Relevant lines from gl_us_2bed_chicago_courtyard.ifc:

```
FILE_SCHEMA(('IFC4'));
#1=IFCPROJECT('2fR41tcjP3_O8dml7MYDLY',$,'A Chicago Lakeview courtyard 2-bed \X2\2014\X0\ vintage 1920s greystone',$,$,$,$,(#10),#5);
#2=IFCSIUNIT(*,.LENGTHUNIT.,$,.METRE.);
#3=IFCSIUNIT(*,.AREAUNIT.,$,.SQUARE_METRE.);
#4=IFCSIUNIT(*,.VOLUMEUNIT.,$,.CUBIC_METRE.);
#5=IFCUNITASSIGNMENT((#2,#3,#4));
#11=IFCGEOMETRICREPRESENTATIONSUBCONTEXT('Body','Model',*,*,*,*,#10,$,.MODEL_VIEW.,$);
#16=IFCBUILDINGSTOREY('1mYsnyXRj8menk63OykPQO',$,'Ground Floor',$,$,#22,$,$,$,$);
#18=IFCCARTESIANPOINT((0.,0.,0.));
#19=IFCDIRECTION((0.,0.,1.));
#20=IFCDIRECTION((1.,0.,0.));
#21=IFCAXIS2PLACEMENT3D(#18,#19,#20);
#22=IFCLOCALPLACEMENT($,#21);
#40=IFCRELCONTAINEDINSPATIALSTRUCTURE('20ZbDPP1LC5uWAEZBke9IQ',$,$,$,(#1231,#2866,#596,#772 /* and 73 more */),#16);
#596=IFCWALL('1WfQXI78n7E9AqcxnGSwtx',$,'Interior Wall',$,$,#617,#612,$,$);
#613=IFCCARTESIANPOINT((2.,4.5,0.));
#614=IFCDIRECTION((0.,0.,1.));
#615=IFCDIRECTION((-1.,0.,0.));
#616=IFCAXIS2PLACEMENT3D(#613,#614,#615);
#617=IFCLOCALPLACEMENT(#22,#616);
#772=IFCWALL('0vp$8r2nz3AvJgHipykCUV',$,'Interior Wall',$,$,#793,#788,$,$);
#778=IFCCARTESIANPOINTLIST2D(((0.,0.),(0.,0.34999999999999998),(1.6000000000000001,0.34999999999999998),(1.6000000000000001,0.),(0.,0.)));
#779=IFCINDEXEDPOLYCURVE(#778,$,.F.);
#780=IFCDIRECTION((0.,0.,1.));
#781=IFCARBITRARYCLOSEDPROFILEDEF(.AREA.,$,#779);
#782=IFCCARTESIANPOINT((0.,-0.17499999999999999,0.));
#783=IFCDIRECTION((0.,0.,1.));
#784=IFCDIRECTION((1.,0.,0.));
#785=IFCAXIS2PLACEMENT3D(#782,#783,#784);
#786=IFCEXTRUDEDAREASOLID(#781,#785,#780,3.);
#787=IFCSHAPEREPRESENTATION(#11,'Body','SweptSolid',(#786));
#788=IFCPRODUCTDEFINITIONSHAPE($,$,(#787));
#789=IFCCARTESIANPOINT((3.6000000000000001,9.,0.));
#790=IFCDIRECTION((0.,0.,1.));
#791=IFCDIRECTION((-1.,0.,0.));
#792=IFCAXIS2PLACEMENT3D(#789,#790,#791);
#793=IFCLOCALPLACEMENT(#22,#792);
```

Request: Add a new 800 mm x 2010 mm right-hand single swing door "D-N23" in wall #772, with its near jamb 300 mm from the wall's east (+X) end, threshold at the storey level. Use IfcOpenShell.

```python
import numpy as np
import ifcopenshell
import ifcopenshell.api.feature
import ifcopenshell.api.geometry
import ifcopenshell.api.root
import ifcopenshell.api.spatial
import ifcopenshell.geom
import ifcopenshell.util.element
import ifcopenshell.util.placement
import ifcopenshell.util.representation
import ifcopenshell.util.shape
import ifcopenshell.util.unit

model = ifcopenshell.open("gl_us_2bed_chicago_courtyard.ifc")
unit_scale = ifcopenshell.util.unit.calculate_unit_scale(model)
settings = ifcopenshell.geom.settings()


def volume(element):
    """Net volume in cubic metres, openings subtracted."""
    shape = ifcopenshell.geom.create_shape(settings, element)
    return ifcopenshell.util.shape.get_volume(shape.geometry)


wall = model.by_guid("0vp$8r2nz3AvJgHipykCUV")
storey = ifcopenshell.util.element.get_container(wall, ifc_class="IfcBuildingStorey")
context = ifcopenshell.util.representation.get_context(model, "Model", "Body", "MODEL_VIEW")
before = volume(wall)

width, height, from_end, sill = 0.8, 2.01, 0.3, 0.0  # metres

# The wall runs along its own X axis, and the end named is its -X end.
wall_shape = ifcopenshell.geom.create_shape(settings, wall)
x, y, z = ifcopenshell.util.shape.get_vertices(wall_shape.geometry).T
start = x.min() + from_end
face, thickness = float(y.min()), float(y.max() - y.min())
wall_matrix = ifcopenshell.util.placement.get_local_placement(wall.ObjectPlacement)
level = ifcopenshell.util.placement.get_local_placement(storey.ObjectPlacement)[2, 3]


def in_wall(x, y):
    """Placement at x, y metres in the wall's axes, at sill height."""
    matrix = wall_matrix.copy()
    matrix[:, 3] = wall_matrix @ np.array([x / unit_scale, y / unit_scale, 0.0, 1.0])
    matrix[2, 3] = level + sill / unit_scale
    return matrix


# Opening: a box that overshoots both wall faces by 50 mm.
opening = ifcopenshell.api.root.create_entity(model, ifc_class="IfcOpeningElement", predefined_type="OPENING")
box = ifcopenshell.api.geometry.add_wall_representation(
    model, context=context, length=width, height=height, thickness=thickness + 0.1
)
ifcopenshell.api.geometry.assign_representation(model, product=opening, representation=box)
ifcopenshell.api.geometry.edit_object_placement(model, product=opening, matrix=in_wall(start, face - 0.05), is_si=False)
ifcopenshell.api.feature.add_feature(model, feature=opening, element=wall)

door = ifcopenshell.api.root.create_entity(model, ifc_class="IfcDoor", name="D-N23", predefined_type="DOOR")
door.OverallWidth, door.OverallHeight = width / unit_scale, height / unit_scale
door.OperationType = "SINGLE_SWING_RIGHT"
body = ifcopenshell.api.geometry.add_door_representation(
    model,
    context=context,
    overall_width=door.OverallWidth,
    overall_height=door.OverallHeight,
    operation_type="SINGLE_SWING_RIGHT",
    lining_properties={"LiningDepth": thickness / unit_scale, "ThresholdDepth": thickness / unit_scale},
)
ifcopenshell.api.geometry.assign_representation(model, product=door, representation=body)
ifcopenshell.api.spatial.assign_container(model, products=[door], relating_structure=storey)
ifcopenshell.api.feature.add_filling(model, opening=opening, element=door)

# The lining spans the wall, so the door starts at the wall face.
ifcopenshell.api.geometry.edit_object_placement(model, product=door, matrix=in_wall(start, face), is_si=False)

after = volume(wall)

print(f"wall volume {before:.3f} -> {after:.3f} m3")

model.write("gl_us_2bed_chicago_courtyard-out.ifc")
```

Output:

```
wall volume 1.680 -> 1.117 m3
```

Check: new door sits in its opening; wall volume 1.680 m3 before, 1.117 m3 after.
